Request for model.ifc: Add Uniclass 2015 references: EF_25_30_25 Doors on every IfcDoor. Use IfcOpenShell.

First a look at what the model holds.

```python
import ifcopenshell

model = ifcopenshell.open("model.ifc")
print(model.schema)
print("classifications:", [c.Name for c in model.by_type("IfcClassification")])
for ifc_class in ("IfcDoor", "IfcRoof", "IfcStair", "IfcWall", "IfcWindow"):
    print(ifc_class, len(model.by_type(ifc_class)))
```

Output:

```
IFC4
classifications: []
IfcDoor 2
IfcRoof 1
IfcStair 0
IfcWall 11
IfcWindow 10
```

```python
import ifcopenshell
import ifcopenshell.api.classification

model = ifcopenshell.open("model.ifc")

system = ifcopenshell.api.classification.add_classification(model, classification="Uniclass 2015")

codes = {
    "IfcDoor": ("EF_25_30_25", "Doors"),
}
for ifc_class, (code, name) in codes.items():
    products = model.by_type(ifc_class)
    ifcopenshell.api.classification.add_reference(
        model, products=products, classification=system, identification=code, name=name
    )
    print(code, len(products))

model.write("model_edited.ifc")
```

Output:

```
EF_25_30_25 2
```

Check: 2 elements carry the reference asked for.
